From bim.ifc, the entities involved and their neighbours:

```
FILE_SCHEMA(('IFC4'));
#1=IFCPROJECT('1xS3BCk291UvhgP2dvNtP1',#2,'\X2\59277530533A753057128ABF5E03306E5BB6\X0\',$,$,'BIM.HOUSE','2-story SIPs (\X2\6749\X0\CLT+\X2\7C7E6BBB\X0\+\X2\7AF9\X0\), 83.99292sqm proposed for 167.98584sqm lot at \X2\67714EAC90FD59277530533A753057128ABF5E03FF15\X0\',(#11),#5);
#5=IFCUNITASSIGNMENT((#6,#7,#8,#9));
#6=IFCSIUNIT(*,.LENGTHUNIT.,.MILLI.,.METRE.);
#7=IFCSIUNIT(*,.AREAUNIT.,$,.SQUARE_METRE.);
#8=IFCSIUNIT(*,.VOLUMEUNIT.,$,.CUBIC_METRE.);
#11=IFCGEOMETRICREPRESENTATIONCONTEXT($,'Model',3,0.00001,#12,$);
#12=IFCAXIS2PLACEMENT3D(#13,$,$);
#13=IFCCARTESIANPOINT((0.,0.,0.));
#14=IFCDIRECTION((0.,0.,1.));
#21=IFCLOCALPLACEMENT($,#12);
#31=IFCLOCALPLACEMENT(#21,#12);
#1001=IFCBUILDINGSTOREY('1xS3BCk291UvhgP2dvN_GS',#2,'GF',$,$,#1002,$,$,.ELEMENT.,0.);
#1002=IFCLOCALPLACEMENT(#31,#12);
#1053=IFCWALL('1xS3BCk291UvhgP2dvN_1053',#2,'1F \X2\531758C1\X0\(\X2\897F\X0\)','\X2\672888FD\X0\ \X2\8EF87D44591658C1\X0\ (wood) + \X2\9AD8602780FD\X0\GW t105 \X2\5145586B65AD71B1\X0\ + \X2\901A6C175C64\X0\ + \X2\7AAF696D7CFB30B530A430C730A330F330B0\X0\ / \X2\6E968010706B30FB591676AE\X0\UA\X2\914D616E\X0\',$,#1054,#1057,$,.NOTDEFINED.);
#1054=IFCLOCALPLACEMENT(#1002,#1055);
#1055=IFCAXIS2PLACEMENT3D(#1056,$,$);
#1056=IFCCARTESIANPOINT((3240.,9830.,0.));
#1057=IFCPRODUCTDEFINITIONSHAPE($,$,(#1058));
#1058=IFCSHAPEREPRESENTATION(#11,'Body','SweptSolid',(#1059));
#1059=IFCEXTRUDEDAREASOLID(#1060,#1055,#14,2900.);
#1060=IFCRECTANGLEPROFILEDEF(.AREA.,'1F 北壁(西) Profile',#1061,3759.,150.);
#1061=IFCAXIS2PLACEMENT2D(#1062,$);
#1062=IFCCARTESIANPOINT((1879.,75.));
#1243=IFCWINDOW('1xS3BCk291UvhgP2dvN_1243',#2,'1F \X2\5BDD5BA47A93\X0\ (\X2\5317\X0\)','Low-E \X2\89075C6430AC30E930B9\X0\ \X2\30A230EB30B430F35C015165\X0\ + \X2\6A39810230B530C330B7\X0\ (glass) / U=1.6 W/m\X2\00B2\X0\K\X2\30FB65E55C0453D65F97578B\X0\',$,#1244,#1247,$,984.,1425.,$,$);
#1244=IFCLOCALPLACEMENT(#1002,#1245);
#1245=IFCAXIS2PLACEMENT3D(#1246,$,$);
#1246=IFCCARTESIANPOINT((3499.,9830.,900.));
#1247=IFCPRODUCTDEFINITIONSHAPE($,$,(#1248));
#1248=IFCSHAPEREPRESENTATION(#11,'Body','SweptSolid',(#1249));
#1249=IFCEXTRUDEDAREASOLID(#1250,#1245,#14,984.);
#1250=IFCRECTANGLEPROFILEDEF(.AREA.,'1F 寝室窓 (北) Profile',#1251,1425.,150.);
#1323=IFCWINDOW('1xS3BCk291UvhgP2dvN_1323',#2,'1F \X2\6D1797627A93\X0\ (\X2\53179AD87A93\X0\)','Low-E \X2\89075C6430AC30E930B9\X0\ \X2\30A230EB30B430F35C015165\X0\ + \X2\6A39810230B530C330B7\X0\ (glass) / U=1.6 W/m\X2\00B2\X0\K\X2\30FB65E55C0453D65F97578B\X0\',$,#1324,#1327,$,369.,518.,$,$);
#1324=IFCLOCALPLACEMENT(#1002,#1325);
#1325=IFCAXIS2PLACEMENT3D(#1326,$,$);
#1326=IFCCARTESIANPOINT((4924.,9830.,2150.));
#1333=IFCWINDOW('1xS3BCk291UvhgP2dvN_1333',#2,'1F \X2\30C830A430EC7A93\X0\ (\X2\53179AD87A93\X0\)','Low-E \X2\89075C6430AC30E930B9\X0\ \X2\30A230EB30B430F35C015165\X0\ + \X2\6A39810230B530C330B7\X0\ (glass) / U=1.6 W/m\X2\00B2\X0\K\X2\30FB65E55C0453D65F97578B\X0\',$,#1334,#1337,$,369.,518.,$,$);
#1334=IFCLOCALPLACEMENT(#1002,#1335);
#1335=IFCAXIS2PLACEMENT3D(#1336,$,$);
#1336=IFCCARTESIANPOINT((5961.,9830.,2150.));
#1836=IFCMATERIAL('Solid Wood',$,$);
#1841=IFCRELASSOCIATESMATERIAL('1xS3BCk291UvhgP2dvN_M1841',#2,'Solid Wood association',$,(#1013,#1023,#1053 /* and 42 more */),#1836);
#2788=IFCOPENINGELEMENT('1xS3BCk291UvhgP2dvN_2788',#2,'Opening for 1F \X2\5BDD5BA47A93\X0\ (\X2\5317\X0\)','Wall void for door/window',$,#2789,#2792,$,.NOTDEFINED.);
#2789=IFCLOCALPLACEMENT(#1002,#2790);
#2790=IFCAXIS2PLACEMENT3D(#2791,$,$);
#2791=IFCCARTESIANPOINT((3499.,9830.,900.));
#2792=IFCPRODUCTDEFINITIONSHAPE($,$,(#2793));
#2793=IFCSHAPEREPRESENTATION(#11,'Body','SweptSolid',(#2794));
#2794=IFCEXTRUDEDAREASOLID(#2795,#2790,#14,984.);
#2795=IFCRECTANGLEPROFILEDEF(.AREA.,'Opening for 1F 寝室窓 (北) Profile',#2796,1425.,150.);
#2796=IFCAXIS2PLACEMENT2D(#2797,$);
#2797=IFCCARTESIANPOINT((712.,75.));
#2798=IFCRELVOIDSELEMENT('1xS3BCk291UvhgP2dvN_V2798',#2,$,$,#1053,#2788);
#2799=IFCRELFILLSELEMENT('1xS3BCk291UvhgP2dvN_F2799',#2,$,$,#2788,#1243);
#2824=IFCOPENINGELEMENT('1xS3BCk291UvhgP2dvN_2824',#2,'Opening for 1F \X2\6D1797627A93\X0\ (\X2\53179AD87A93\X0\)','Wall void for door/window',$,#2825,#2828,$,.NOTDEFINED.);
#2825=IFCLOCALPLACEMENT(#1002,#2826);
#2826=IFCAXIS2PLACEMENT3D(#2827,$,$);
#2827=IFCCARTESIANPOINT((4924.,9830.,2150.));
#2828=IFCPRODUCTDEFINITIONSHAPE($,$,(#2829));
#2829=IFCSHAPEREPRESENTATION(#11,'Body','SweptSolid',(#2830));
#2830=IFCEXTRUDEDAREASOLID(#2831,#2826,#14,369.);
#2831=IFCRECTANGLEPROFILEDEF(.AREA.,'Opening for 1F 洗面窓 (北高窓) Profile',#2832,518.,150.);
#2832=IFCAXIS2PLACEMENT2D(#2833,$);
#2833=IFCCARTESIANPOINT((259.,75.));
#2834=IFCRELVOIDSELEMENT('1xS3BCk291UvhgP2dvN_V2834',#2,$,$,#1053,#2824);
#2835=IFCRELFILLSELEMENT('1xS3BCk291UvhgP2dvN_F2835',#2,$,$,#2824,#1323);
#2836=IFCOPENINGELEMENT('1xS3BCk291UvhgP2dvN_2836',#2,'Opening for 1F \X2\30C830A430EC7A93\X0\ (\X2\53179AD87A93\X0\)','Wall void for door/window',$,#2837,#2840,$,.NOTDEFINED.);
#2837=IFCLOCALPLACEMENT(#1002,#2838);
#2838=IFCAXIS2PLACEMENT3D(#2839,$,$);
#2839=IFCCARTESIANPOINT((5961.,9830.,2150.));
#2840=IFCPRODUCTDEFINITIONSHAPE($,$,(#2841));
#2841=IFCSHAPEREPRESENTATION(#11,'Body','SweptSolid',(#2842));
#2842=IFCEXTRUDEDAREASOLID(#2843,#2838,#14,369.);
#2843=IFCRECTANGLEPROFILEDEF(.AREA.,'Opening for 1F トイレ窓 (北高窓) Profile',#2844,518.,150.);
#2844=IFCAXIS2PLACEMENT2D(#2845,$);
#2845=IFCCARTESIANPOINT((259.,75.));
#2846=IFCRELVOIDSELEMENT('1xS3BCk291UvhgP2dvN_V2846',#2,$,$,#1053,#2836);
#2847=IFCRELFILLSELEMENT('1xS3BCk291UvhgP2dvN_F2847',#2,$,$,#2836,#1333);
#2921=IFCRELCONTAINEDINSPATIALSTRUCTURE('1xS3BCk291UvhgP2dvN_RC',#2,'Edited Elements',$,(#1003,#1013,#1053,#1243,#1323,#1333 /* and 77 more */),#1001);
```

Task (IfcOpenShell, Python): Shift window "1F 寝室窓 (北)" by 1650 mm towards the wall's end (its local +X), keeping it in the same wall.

```python
import ifcopenshell
import ifcopenshell.api.geometry
import ifcopenshell.util.placement
import ifcopenshell.util.unit

model = ifcopenshell.open("bim.ifc")
unit_scale = ifcopenshell.util.unit.calculate_unit_scale(model)

window = model.by_guid("1xS3BCk291UvhgP2dvN_1243")
opening = window.FillsVoids[0].RelatingOpeningElement
wall = opening.VoidsElements[0].RelatingBuildingElement

wall_matrix = ifcopenshell.util.placement.get_local_placement(wall.ObjectPlacement)
shift = wall_matrix[:3, 0] * 1.65 / unit_scale
before = ifcopenshell.util.placement.get_local_placement(window.ObjectPlacement)[:3, 3].copy()

# The window is not placed relative to its opening, so move both.
for product in (opening, window):
    matrix = ifcopenshell.util.placement.get_local_placement(product.ObjectPlacement)
    matrix[:3, 3] += shift
    ifcopenshell.api.geometry.edit_object_placement(model, product=product, matrix=matrix, is_si=False)

after = ifcopenshell.util.placement.get_local_placement(window.ObjectPlacement)[:3, 3]
print("window moved by", (after - before).round(3) + 0.0)

model.write("bim_updated.ifc")
```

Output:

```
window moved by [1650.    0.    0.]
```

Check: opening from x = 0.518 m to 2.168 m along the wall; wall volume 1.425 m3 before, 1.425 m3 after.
